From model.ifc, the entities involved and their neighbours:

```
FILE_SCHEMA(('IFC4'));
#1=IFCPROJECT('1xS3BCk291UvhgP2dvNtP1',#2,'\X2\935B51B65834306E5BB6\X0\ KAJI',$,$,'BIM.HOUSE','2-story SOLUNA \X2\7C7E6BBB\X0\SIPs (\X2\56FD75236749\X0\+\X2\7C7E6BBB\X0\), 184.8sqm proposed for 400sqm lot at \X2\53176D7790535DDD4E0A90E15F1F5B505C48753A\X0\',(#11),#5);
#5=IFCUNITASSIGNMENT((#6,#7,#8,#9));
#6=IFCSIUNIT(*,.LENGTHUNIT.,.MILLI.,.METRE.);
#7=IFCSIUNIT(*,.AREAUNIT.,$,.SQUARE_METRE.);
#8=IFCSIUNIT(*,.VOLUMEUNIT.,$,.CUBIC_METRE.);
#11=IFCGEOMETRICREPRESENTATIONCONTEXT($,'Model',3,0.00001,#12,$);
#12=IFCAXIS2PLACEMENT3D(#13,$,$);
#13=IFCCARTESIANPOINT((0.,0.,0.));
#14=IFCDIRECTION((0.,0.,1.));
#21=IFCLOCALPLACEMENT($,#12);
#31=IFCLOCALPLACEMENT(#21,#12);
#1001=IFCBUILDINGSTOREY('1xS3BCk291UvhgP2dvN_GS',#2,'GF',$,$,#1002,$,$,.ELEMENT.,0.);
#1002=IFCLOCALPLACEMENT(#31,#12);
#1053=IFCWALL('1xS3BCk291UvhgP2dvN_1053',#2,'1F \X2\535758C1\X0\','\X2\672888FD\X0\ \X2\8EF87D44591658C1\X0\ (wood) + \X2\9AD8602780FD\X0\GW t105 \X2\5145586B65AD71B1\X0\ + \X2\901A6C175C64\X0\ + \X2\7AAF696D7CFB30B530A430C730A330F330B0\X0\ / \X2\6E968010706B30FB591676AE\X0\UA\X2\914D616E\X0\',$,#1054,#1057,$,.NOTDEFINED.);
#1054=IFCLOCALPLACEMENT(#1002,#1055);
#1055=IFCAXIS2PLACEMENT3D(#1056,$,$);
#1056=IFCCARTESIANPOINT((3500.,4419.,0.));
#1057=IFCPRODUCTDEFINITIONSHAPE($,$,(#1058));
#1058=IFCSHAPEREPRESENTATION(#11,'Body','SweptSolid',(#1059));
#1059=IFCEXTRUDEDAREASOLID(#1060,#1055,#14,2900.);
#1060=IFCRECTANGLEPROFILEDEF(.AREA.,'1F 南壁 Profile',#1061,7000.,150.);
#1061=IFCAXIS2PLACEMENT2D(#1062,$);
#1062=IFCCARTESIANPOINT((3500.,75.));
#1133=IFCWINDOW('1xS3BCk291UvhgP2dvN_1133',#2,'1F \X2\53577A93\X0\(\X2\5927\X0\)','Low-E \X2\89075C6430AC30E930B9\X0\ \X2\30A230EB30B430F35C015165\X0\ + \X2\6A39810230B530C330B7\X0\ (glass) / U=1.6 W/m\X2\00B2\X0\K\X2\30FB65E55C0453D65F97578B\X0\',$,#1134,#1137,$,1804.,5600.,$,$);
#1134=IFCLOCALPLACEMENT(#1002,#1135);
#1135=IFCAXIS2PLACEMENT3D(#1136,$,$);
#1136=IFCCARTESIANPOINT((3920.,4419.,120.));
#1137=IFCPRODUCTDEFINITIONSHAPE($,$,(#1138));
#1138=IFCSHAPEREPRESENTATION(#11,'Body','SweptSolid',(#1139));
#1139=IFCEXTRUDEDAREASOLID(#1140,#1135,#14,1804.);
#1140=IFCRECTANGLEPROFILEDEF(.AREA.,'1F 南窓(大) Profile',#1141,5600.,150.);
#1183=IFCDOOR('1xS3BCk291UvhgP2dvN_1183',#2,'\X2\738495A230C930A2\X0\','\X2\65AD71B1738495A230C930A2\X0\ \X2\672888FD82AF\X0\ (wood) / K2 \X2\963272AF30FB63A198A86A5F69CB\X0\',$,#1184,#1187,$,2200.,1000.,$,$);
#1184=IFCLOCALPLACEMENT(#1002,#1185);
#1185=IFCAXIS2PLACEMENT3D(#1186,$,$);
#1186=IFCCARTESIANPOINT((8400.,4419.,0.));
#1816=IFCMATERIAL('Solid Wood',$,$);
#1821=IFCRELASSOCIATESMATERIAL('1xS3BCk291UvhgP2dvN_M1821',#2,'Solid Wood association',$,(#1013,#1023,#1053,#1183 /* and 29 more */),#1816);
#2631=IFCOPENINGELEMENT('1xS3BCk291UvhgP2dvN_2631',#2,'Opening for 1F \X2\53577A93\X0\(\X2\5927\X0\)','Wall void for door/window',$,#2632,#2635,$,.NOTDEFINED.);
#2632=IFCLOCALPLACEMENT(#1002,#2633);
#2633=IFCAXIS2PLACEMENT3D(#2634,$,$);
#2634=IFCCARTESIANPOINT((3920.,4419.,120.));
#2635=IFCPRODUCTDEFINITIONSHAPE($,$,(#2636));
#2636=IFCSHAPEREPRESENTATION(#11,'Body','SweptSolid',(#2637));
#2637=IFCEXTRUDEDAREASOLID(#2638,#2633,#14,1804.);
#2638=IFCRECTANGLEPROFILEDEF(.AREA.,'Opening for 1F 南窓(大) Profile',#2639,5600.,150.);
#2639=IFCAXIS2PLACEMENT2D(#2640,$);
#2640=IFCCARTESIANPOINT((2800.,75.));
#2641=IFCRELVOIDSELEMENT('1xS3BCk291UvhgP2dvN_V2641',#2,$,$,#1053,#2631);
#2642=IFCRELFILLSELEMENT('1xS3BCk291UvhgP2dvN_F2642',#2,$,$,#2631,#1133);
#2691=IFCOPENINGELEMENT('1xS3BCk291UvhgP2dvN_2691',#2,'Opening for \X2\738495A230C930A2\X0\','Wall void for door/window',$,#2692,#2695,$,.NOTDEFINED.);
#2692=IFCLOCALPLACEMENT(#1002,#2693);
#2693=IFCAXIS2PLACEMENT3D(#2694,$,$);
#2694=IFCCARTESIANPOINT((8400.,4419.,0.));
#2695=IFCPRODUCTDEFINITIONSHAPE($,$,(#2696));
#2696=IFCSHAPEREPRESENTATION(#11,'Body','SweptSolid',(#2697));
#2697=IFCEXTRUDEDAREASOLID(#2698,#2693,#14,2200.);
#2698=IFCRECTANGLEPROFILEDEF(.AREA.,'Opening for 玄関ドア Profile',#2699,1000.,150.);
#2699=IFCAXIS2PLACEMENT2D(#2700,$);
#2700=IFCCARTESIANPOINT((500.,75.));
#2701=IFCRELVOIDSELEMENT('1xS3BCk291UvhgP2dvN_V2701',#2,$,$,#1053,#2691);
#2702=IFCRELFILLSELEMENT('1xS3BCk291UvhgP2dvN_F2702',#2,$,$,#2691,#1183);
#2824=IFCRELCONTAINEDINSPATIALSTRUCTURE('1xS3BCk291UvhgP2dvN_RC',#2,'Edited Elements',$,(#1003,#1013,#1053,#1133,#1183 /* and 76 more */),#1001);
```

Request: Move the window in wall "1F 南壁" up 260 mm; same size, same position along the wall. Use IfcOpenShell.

```python
import numpy as np
import ifcopenshell
import ifcopenshell.api.geometry
import ifcopenshell.util.placement
import ifcopenshell.util.unit

model = ifcopenshell.open("model.ifc")
unit_scale = ifcopenshell.util.unit.calculate_unit_scale(model)

window = model.by_guid("1xS3BCk291UvhgP2dvN_1133")
opening = window.FillsVoids[0].RelatingOpeningElement
dz = 0.26 / unit_scale

shift = np.array([0.0, 0.0, dz])
# The window is not placed relative to its opening, so move both.
for product in (opening, window):
    matrix = ifcopenshell.util.placement.get_local_placement(product.ObjectPlacement)
    matrix[:3, 3] += shift
    ifcopenshell.api.geometry.edit_object_placement(model, product=product, matrix=matrix, is_si=False)

print(f"moved by {dz * unit_scale:+.3f} m")

model.write("model-out.ifc")
```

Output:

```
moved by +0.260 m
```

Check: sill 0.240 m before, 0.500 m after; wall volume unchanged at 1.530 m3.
